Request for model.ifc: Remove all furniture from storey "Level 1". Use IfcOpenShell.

First a look at what the model holds.

```python
import ifcopenshell
import ifcopenshell.util.element

model = ifcopenshell.open("model.ifc")
print(model.schema)
storey = next(s for s in model.by_type("IfcBuildingStorey") if s.Name == "Level 1")
furniture = [e for e in ifcopenshell.util.element.get_decomposition(storey) if e.is_a("IfcFurnishingElement")]
seen = {}
for e in furniture:
    element_type = ifcopenshell.util.element.get_type(e)
    name = element_type.Name if element_type not in (None, e) else None
    seen[name] = seen.get(name, 0) + 1
for name, count in sorted(seen.items(), key=str):
    print(count, "x", name)
```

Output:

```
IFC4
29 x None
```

```python
import ifcopenshell
import ifcopenshell.api.root
import ifcopenshell.util.element

model = ifcopenshell.open("model.ifc")

storey = next(s for s in model.by_type("IfcBuildingStorey") if s.Name == "Level 1")
furniture = [e for e in ifcopenshell.util.element.get_decomposition(storey) if e.is_a("IfcFurnishingElement")]

for e in furniture:
    ifcopenshell.api.root.remove_product(model, product=e)
print(len(furniture), "removed")

model.write("model_rev.ifc")
```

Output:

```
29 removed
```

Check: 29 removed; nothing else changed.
